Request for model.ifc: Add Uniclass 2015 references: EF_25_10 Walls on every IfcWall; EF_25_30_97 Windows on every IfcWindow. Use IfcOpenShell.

First a look at what the model holds.

```python
import ifcopenshell

model = ifcopenshell.open("model.ifc")
print(model.schema)
print("classifications:", [c.Name for c in model.by_type("IfcClassification")])
for ifc_class in ("IfcDoor", "IfcRoof", "IfcStair", "IfcWall", "IfcWindow"):
    print(ifc_class, len(model.by_type(ifc_class)))
```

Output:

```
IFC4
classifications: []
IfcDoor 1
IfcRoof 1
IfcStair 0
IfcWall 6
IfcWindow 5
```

```python
import ifcopenshell
import ifcopenshell.api.classification

model = ifcopenshell.open("model.ifc")

system = ifcopenshell.api.classification.add_classification(model, classification="Uniclass 2015")

codes = {
    "IfcWall": ("EF_25_10", "Walls"),
    "IfcWindow": ("EF_25_30_97", "Windows"),
}
for ifc_class, (code, name) in codes.items():
    products = model.by_type(ifc_class)
    ifcopenshell.api.classification.add_reference(
        model, products=products, classification=system, identification=code, name=name
    )
    print(code, len(products))

model.write("model_updated.ifc")
```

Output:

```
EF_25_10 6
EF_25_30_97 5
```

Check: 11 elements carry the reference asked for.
